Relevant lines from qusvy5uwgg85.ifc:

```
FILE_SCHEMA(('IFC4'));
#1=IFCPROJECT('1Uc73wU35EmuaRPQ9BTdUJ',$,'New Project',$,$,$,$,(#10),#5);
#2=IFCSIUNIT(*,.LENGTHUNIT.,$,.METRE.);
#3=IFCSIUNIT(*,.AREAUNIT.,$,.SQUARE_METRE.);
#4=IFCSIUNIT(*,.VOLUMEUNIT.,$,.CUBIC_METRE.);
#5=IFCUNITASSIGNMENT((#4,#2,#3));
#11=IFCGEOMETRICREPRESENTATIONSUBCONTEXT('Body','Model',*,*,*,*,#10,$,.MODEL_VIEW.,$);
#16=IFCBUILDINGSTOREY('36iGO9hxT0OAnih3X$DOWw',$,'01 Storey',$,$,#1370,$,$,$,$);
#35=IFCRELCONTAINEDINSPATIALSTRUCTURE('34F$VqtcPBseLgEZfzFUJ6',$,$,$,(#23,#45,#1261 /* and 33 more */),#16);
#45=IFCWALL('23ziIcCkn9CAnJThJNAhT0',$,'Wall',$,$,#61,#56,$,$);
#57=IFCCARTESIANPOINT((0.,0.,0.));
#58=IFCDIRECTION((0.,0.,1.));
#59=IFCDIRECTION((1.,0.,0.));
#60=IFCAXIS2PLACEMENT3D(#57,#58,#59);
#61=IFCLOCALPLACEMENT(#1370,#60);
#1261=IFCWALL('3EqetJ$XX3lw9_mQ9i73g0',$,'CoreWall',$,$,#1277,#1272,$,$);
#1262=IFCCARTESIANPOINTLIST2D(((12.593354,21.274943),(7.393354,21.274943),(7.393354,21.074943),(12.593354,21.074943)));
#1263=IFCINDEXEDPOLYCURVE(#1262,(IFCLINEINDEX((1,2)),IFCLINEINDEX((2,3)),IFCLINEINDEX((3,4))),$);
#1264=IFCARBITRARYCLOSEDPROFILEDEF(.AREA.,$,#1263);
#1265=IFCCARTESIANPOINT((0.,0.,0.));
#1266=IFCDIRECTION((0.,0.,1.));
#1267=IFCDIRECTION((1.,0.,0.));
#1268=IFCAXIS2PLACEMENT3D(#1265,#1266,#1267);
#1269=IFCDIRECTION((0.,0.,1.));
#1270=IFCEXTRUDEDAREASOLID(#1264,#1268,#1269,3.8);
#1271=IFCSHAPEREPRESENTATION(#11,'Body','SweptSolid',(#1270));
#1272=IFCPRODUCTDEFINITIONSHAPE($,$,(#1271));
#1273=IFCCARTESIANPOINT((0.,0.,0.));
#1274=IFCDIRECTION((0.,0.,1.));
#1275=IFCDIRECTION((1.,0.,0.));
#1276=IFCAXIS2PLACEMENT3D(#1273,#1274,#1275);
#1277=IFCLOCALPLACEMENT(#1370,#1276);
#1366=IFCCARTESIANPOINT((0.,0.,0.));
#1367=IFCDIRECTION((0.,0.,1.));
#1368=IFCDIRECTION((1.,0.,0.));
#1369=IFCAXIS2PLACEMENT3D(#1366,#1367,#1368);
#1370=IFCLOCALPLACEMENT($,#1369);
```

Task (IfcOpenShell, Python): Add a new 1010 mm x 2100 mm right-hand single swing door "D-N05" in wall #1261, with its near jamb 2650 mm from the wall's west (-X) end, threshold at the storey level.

```python
import numpy as np
import ifcopenshell
import ifcopenshell.api.feature
import ifcopenshell.api.geometry
import ifcopenshell.api.root
import ifcopenshell.api.spatial
import ifcopenshell.geom
import ifcopenshell.util.element
import ifcopenshell.util.placement
import ifcopenshell.util.representation
import ifcopenshell.util.shape
import ifcopenshell.util.unit

model = ifcopenshell.open("qusvy5uwgg85.ifc")
unit_scale = ifcopenshell.util.unit.calculate_unit_scale(model)
settings = ifcopenshell.geom.settings()


def volume(element):
    """Net volume in cubic metres, openings subtracted."""
    shape = ifcopenshell.geom.create_shape(settings, element)
    return ifcopenshell.util.shape.get_volume(shape.geometry)


wall = model.by_guid("3EqetJ$XX3lw9_mQ9i73g0")
storey = ifcopenshell.util.element.get_container(wall, ifc_class="IfcBuildingStorey")
context = ifcopenshell.util.representation.get_context(model, "Model", "Body", "MODEL_VIEW")
before = volume(wall)

width, height, from_end, sill = 1.01, 2.1, 2.65, 0.0  # metres

# The wall runs along its own X axis, and the end named is its -X end.
wall_shape = ifcopenshell.geom.create_shape(settings, wall)
x, y, z = ifcopenshell.util.shape.get_vertices(wall_shape.geometry).T
start = x.min() + from_end
face, thickness = float(y.min()), float(y.max() - y.min())
wall_matrix = ifcopenshell.util.placement.get_local_placement(wall.ObjectPlacement)
level = ifcopenshell.util.placement.get_local_placement(storey.ObjectPlacement)[2, 3]


def in_wall(x, y):
    """Placement at x, y metres in the wall's axes, at sill height."""
    matrix = wall_matrix.copy()
    matrix[:, 3] = wall_matrix @ np.array([x / unit_scale, y / unit_scale, 0.0, 1.0])
    matrix[2, 3] = level + sill / unit_scale
    return matrix


# Opening: a box that overshoots both wall faces by 50 mm.
opening = ifcopenshell.api.root.create_entity(model, ifc_class="IfcOpeningElement", predefined_type="OPENING")
box = ifcopenshell.api.geometry.add_wall_representation(
    model, context=context, length=width, height=height, thickness=thickness + 0.1
)
ifcopenshell.api.geometry.assign_representation(model, product=opening, representation=box)
ifcopenshell.api.geometry.edit_object_placement(model, product=opening, matrix=in_wall(start, face - 0.05), is_si=False)
ifcopenshell.api.feature.add_feature(model, feature=opening, element=wall)

door = ifcopenshell.api.root.create_entity(model, ifc_class="IfcDoor", name="D-N05", predefined_type="DOOR")
door.OverallWidth, door.OverallHeight = width / unit_scale, height / unit_scale
door.OperationType = "SINGLE_SWING_RIGHT"
body = ifcopenshell.api.geometry.add_door_representation(
    model,
    context=context,
    overall_width=door.OverallWidth,
    overall_height=door.OverallHeight,
    operation_type="SINGLE_SWING_RIGHT",
    lining_properties={"LiningDepth": thickness / unit_scale, "ThresholdDepth": thickness / unit_scale},
)
ifcopenshell.api.geometry.assign_representation(model, product=door, representation=body)
ifcopenshell.api.spatial.assign_container(model, products=[door], relating_structure=storey)
ifcopenshell.api.feature.add_filling(model, opening=opening, element=door)

# The lining spans the wall, so the door starts at the wall face.
ifcopenshell.api.geometry.edit_object_placement(model, product=door, matrix=in_wall(start, face), is_si=False)

after = volume(wall)

print(f"wall volume {before:.3f} -> {after:.3f} m3")

model.write("qusvy5uwgg85-out.ifc")
```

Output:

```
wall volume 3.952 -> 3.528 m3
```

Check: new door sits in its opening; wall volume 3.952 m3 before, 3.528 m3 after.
